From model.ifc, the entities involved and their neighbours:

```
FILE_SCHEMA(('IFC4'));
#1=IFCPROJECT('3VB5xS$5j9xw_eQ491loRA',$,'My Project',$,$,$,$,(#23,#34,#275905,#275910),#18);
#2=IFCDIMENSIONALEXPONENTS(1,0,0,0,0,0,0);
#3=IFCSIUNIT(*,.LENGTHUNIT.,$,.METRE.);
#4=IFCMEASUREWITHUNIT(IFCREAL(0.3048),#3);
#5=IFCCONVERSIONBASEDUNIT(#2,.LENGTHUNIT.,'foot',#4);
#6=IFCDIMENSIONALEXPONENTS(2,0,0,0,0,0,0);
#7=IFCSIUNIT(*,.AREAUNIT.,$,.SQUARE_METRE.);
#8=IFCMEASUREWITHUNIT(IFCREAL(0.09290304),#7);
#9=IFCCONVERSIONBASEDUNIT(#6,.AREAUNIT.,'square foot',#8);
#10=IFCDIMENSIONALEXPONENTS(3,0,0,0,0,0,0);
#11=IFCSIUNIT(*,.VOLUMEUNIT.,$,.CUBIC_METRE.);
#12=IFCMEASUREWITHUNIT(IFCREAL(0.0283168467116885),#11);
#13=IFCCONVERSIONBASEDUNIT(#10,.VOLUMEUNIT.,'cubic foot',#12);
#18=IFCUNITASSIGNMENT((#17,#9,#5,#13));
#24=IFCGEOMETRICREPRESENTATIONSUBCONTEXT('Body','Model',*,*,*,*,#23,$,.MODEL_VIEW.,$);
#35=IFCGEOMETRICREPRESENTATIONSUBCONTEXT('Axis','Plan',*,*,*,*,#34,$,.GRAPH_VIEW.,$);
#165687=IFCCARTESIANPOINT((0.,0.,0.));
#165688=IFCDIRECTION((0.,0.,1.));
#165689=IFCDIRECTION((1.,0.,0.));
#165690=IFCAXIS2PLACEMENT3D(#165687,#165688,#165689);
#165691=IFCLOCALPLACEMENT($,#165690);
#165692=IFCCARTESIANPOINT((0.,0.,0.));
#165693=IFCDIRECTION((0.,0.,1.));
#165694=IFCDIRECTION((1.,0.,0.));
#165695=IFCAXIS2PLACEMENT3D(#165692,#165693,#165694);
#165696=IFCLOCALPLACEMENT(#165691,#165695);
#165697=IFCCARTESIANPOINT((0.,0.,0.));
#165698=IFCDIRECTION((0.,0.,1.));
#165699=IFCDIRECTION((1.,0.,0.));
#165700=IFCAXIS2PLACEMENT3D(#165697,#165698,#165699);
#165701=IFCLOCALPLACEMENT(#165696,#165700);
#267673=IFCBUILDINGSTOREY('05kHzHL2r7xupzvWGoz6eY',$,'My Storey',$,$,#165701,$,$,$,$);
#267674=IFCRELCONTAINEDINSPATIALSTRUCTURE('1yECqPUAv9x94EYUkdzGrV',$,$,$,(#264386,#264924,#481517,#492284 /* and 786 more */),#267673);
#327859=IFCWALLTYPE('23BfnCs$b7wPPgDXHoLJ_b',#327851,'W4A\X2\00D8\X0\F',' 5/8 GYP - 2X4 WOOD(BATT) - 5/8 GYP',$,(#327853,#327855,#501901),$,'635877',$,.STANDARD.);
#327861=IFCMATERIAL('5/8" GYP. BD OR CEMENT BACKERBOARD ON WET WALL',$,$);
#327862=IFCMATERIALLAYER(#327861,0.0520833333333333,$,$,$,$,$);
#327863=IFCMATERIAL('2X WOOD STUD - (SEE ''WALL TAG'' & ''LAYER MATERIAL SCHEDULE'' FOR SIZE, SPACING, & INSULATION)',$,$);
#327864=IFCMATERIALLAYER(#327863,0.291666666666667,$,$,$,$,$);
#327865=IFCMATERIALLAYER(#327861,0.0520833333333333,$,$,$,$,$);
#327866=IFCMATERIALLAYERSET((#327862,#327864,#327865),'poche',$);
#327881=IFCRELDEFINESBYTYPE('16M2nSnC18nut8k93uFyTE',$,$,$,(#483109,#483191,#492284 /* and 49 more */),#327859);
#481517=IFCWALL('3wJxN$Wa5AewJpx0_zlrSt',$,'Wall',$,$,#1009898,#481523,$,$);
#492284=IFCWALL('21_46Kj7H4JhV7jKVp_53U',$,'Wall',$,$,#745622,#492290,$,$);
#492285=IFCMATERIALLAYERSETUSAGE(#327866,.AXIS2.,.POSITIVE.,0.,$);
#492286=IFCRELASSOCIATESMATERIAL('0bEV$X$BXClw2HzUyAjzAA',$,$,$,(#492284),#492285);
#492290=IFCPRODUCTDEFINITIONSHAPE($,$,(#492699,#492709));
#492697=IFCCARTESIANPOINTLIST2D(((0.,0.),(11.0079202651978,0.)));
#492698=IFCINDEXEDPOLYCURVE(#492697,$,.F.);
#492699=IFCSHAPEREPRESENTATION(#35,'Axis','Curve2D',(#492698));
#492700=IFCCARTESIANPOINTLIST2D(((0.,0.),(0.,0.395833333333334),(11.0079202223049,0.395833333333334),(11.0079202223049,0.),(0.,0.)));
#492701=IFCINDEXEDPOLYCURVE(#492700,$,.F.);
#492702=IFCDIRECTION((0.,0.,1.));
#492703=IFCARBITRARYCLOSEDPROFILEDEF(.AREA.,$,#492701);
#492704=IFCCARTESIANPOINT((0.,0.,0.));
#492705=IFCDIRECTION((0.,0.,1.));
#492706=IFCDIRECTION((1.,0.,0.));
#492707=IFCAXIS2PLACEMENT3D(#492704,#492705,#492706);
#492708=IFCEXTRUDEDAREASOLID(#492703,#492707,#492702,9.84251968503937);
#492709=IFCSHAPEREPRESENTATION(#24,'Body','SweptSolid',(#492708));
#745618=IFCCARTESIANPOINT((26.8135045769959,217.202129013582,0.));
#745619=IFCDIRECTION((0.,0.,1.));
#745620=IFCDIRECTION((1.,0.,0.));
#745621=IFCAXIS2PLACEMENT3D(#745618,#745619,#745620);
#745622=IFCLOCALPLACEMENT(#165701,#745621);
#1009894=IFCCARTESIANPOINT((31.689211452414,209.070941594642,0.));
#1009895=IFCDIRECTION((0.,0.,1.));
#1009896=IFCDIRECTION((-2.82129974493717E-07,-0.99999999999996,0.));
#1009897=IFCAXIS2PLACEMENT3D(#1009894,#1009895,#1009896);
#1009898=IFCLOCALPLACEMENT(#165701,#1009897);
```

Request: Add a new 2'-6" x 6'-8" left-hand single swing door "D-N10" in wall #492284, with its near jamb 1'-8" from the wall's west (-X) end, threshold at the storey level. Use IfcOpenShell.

```python
import numpy as np
import ifcopenshell
import ifcopenshell.api.feature
import ifcopenshell.api.geometry
import ifcopenshell.api.root
import ifcopenshell.api.spatial
import ifcopenshell.geom
import ifcopenshell.util.element
import ifcopenshell.util.placement
import ifcopenshell.util.representation
import ifcopenshell.util.shape
import ifcopenshell.util.unit

model = ifcopenshell.open("model.ifc")
unit_scale = ifcopenshell.util.unit.calculate_unit_scale(model)
settings = ifcopenshell.geom.settings()


def volume(element):
    """Net volume in cubic metres, openings subtracted."""
    shape = ifcopenshell.geom.create_shape(settings, element)
    return ifcopenshell.util.shape.get_volume(shape.geometry)


wall = model.by_guid("21_46Kj7H4JhV7jKVp_53U")
storey = ifcopenshell.util.element.get_container(wall, ifc_class="IfcBuildingStorey")
context = ifcopenshell.util.representation.get_context(model, "Model", "Body", "MODEL_VIEW")
before = volume(wall)

width, height, from_end, sill = 0.762, 2.032, 0.508, 0.0  # metres

# The wall runs along its own X axis, and the end named is its -X end.
wall_shape = ifcopenshell.geom.create_shape(settings, wall)
x, y, z = ifcopenshell.util.shape.get_vertices(wall_shape.geometry).T
start = x.min() + from_end
face, thickness = float(y.min()), float(y.max() - y.min())
wall_matrix = ifcopenshell.util.placement.get_local_placement(wall.ObjectPlacement)
level = ifcopenshell.util.placement.get_local_placement(storey.ObjectPlacement)[2, 3]


def in_wall(x, y):
    """Placement at x, y metres in the wall's axes, at sill height."""
    matrix = wall_matrix.copy()
    matrix[:, 3] = wall_matrix @ np.array([x / unit_scale, y / unit_scale, 0.0, 1.0])
    matrix[2, 3] = level + sill / unit_scale
    return matrix


# Opening: a box that overshoots both wall faces by 50 mm.
opening = ifcopenshell.api.root.create_entity(model, ifc_class="IfcOpeningElement", predefined_type="OPENING")
box = ifcopenshell.api.geometry.add_wall_representation(
    model, context=context, length=width, height=height, thickness=thickness + 0.1
)
ifcopenshell.api.geometry.assign_representation(model, product=opening, representation=box)
ifcopenshell.api.geometry.edit_object_placement(model, product=opening, matrix=in_wall(start, face - 0.05), is_si=False)
ifcopenshell.api.feature.add_feature(model, feature=opening, element=wall)

door = ifcopenshell.api.root.create_entity(model, ifc_class="IfcDoor", name="D-N10", predefined_type="DOOR")
door.OverallWidth, door.OverallHeight = width / unit_scale, height / unit_scale
door.OperationType = "SINGLE_SWING_LEFT"
body = ifcopenshell.api.geometry.add_door_representation(
    model,
    context=context,
    overall_width=door.OverallWidth,
    overall_height=door.OverallHeight,
    operation_type="SINGLE_SWING_LEFT",
    lining_properties={"LiningDepth": thickness / unit_scale, "ThresholdDepth": thickness / unit_scale},
)
ifcopenshell.api.geometry.assign_representation(model, product=door, representation=body)
ifcopenshell.api.spatial.assign_container(model, products=[door], relating_structure=storey)
ifcopenshell.api.feature.add_filling(model, opening=opening, element=door)

# The lining spans the wall, so the door starts at the wall face.
ifcopenshell.api.geometry.edit_object_placement(model, product=door, matrix=in_wall(start, face), is_si=False)

after = volume(wall)

print(f"wall volume {before:.3f} -> {after:.3f} m3")

model.write("model_edited.ifc")
```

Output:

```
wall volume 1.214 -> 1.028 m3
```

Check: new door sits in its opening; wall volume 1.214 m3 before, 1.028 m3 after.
